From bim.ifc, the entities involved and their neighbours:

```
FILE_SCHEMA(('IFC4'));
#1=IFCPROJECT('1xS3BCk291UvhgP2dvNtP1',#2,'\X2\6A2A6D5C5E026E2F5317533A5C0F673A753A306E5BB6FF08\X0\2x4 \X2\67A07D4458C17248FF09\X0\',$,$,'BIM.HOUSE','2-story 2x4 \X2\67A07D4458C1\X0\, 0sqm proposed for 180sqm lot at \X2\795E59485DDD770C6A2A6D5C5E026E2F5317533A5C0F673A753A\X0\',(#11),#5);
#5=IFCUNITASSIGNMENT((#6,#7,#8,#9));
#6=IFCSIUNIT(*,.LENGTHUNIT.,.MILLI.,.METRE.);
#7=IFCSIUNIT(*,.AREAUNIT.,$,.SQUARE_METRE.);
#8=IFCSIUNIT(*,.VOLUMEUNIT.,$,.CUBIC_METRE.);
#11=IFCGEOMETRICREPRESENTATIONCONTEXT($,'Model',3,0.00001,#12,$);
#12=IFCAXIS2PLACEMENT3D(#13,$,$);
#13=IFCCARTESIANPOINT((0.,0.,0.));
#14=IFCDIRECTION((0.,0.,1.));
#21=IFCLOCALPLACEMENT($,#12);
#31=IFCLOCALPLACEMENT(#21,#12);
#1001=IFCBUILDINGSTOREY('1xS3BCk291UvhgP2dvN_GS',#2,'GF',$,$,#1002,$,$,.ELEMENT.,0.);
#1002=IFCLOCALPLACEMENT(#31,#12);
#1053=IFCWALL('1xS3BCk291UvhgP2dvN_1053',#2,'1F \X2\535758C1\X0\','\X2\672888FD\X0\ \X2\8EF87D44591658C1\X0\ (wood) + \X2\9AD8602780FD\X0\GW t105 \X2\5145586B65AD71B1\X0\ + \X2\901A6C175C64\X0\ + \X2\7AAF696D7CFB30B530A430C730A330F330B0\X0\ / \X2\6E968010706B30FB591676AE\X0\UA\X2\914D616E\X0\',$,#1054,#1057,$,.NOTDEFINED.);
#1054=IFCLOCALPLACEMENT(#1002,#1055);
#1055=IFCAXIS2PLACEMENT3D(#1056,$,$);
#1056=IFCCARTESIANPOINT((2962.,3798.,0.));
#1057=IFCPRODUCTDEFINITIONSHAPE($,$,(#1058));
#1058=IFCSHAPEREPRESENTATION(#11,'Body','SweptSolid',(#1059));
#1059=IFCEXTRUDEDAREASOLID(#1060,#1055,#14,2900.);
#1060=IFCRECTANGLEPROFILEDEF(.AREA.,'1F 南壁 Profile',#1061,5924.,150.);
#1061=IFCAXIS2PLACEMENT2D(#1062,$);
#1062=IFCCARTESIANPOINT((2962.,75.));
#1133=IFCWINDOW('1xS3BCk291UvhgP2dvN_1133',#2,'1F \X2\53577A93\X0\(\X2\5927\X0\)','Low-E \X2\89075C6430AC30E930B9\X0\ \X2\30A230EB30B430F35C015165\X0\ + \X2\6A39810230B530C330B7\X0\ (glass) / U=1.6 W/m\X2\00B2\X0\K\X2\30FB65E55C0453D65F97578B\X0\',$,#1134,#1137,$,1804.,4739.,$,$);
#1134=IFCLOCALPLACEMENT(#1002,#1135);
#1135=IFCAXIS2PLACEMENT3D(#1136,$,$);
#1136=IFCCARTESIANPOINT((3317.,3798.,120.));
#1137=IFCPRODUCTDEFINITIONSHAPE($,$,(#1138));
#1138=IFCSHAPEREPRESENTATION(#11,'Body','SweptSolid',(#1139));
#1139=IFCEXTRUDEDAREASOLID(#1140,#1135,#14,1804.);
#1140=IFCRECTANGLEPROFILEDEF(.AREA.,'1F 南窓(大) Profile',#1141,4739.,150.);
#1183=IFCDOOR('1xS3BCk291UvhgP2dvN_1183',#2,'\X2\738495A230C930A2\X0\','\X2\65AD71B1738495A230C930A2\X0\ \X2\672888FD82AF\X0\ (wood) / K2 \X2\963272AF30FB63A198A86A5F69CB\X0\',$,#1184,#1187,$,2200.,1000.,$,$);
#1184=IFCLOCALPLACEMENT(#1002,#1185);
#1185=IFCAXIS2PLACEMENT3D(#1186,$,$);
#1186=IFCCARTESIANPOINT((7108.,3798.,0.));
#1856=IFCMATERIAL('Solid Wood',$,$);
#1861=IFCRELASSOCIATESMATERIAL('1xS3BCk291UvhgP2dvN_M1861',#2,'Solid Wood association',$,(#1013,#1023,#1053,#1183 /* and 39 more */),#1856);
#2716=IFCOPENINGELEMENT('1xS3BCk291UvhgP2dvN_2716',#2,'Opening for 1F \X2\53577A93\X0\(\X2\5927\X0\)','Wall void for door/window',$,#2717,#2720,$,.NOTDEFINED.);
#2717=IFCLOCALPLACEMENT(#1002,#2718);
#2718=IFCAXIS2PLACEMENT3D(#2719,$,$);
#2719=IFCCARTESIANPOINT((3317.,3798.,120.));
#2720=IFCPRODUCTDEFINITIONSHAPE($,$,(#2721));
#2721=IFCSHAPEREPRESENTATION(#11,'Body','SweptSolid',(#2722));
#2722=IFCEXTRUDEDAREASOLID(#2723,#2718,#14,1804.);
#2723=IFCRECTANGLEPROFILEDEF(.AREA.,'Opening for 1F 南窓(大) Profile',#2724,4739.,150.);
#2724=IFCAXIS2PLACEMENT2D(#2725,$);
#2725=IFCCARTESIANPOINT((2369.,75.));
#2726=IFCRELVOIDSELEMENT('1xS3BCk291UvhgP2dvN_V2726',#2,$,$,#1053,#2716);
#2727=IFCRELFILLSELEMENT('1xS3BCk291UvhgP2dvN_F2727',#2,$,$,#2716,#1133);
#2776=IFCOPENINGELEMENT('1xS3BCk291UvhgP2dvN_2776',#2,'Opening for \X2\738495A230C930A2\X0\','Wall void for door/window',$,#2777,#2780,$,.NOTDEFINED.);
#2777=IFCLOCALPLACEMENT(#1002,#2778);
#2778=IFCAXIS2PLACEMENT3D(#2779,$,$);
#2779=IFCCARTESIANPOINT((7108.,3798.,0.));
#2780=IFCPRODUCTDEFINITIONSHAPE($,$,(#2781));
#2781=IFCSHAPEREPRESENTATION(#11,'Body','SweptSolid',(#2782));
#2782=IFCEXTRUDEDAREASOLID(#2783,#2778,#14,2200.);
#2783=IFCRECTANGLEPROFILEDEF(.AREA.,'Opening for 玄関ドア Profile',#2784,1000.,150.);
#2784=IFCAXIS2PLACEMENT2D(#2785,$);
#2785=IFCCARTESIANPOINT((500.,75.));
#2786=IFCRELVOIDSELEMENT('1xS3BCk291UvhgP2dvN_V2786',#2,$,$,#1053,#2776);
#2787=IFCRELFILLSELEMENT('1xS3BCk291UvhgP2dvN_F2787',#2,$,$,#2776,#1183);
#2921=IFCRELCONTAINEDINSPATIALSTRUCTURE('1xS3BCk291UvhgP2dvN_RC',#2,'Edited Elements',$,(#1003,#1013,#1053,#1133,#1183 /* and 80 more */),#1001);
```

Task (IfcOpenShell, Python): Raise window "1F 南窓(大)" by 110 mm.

```python
import numpy as np
import ifcopenshell
import ifcopenshell.api.geometry
import ifcopenshell.util.placement
import ifcopenshell.util.unit

model = ifcopenshell.open("bim.ifc")
unit_scale = ifcopenshell.util.unit.calculate_unit_scale(model)

window = model.by_guid("1xS3BCk291UvhgP2dvN_1133")
opening = window.FillsVoids[0].RelatingOpeningElement
dz = 0.11 / unit_scale

shift = np.array([0.0, 0.0, dz])
# The window is not placed relative to its opening, so move both.
for product in (opening, window):
    matrix = ifcopenshell.util.placement.get_local_placement(product.ObjectPlacement)
    matrix[:3, 3] += shift
    ifcopenshell.api.geometry.edit_object_placement(model, product=product, matrix=matrix, is_si=False)

print(f"moved by {dz * unit_scale:+.3f} m")

model.write("bim_edited.ifc")
```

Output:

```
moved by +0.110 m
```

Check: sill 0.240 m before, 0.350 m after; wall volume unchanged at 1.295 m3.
